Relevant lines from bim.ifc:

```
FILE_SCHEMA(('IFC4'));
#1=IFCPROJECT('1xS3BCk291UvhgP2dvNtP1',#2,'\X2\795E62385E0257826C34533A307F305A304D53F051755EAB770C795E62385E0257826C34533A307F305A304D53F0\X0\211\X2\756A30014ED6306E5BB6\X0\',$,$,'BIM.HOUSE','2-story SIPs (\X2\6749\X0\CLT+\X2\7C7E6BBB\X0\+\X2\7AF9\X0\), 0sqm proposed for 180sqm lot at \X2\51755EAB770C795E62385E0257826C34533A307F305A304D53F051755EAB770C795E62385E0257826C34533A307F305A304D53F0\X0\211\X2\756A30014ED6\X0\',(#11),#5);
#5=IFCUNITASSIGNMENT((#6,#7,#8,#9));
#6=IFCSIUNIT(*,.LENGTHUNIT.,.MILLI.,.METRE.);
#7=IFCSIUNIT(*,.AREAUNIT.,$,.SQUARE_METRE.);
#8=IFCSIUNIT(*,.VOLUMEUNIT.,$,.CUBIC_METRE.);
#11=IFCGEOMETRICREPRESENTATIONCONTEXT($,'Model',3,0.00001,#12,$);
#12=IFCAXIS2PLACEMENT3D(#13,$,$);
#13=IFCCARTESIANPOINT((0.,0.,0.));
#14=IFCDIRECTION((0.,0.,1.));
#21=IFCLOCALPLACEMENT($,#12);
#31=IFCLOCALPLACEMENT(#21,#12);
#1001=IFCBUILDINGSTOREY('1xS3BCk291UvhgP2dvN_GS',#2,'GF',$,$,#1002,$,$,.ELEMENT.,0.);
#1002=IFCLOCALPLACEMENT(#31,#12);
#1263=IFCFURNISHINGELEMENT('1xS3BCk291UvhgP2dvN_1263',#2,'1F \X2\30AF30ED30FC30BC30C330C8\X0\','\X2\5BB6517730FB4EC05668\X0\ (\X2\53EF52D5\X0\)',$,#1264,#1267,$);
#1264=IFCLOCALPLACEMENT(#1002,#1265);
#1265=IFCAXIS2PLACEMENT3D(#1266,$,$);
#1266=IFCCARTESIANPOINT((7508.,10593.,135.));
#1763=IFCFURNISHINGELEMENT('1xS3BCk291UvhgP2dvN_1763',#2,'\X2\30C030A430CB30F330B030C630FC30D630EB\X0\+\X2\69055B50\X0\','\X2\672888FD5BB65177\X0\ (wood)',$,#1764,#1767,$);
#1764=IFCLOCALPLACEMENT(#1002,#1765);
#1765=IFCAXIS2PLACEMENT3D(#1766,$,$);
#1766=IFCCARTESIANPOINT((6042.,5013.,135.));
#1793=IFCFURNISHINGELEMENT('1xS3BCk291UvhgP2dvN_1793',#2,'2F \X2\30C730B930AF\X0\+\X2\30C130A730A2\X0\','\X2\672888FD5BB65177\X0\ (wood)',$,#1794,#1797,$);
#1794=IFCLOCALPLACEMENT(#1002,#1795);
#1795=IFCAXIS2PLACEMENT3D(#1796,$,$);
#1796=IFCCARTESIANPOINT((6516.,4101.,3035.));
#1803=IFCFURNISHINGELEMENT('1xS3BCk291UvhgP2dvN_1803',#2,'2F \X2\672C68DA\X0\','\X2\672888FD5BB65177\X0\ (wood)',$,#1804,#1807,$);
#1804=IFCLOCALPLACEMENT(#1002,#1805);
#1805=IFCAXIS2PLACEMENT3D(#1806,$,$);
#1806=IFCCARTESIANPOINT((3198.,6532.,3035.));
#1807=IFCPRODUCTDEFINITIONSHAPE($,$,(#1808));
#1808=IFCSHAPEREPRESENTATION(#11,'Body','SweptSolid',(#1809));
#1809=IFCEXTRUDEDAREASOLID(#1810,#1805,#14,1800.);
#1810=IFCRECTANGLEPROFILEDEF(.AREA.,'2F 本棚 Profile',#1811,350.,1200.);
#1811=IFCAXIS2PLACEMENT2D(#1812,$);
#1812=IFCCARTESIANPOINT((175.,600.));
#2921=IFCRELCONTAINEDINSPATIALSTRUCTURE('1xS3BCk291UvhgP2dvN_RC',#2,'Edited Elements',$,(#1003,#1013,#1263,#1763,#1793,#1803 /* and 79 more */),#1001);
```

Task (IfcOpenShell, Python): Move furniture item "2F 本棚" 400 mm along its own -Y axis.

```python
import ifcopenshell
import ifcopenshell.api.geometry
import ifcopenshell.util.placement

model = ifcopenshell.open("bim.ifc")

item = model.by_guid("1xS3BCk291UvhgP2dvN_1803")
matrix = ifcopenshell.util.placement.get_local_placement(item.ObjectPlacement)
matrix[:3, 3] -= matrix[:3, 1] * 400.0
ifcopenshell.api.geometry.edit_object_placement(model, product=item, matrix=matrix, is_si=False)

print(ifcopenshell.util.placement.get_local_placement(item.ObjectPlacement).round(3) + 0.0)

model.write("bim_updated.ifc")
```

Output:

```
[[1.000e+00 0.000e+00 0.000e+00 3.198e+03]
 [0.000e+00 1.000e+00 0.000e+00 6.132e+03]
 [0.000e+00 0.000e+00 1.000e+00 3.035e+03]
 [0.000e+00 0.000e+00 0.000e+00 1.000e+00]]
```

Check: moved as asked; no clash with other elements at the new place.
